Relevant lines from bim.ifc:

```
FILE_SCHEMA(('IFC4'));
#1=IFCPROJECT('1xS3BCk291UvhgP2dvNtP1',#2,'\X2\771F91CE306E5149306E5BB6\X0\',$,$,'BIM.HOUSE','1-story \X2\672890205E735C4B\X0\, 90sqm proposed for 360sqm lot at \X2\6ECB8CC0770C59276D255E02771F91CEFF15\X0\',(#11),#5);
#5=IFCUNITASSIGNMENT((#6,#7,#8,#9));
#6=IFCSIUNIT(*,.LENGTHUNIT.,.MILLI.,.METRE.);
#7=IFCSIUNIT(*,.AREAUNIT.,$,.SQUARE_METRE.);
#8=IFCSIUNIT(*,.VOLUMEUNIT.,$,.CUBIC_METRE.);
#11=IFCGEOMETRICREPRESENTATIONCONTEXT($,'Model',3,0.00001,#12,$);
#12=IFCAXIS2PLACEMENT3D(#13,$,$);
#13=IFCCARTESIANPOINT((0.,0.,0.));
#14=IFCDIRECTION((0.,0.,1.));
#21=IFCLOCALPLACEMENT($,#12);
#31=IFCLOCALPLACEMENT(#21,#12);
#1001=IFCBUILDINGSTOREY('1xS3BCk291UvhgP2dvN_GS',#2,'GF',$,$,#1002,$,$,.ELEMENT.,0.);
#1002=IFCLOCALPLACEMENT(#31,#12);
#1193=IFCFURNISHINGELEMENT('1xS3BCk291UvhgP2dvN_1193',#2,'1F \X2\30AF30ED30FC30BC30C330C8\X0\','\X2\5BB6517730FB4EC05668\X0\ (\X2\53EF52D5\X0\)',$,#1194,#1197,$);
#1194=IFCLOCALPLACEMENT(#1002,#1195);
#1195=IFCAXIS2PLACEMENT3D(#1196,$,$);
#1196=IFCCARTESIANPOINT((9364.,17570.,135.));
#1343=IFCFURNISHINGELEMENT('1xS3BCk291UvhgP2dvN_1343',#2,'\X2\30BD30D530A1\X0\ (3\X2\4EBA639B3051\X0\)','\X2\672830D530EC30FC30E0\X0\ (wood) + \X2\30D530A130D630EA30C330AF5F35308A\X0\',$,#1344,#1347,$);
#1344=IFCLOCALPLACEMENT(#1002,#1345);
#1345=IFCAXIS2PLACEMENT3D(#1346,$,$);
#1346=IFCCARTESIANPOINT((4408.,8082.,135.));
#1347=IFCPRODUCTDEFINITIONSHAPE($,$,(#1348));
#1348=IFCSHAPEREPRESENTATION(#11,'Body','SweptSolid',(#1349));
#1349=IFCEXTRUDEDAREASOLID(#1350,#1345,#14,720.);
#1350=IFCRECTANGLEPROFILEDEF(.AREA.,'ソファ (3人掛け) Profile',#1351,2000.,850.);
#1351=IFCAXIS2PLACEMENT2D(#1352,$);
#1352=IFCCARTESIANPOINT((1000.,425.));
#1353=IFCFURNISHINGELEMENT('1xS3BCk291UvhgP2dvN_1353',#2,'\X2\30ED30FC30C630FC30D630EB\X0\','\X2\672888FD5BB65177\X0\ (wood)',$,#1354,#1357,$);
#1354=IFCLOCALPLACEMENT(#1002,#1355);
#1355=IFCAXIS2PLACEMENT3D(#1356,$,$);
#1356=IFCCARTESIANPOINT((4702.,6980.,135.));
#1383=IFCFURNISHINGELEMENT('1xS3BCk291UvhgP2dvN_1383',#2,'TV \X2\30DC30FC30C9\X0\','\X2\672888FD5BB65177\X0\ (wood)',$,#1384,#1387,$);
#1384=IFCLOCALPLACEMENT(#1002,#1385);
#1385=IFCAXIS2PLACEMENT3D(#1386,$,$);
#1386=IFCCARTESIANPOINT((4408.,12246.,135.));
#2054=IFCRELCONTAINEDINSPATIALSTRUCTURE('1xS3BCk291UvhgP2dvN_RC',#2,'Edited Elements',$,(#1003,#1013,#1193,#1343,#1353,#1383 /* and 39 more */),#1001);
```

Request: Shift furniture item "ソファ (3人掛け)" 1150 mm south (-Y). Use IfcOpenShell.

```python
import ifcopenshell
import ifcopenshell.api.geometry
import ifcopenshell.util.placement

model = ifcopenshell.open("bim.ifc")

item = model.by_guid("1xS3BCk291UvhgP2dvN_1343")
matrix = ifcopenshell.util.placement.get_local_placement(item.ObjectPlacement)
matrix[1, 3] -= 1150.0
ifcopenshell.api.geometry.edit_object_placement(model, product=item, matrix=matrix, is_si=False)

print(ifcopenshell.util.placement.get_local_placement(item.ObjectPlacement).round(3) + 0.0)

model.write("bim-out.ifc")
```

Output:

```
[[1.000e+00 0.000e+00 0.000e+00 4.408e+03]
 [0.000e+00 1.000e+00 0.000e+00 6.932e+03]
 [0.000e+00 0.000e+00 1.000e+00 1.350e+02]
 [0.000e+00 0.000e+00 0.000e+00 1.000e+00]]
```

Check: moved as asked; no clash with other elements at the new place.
